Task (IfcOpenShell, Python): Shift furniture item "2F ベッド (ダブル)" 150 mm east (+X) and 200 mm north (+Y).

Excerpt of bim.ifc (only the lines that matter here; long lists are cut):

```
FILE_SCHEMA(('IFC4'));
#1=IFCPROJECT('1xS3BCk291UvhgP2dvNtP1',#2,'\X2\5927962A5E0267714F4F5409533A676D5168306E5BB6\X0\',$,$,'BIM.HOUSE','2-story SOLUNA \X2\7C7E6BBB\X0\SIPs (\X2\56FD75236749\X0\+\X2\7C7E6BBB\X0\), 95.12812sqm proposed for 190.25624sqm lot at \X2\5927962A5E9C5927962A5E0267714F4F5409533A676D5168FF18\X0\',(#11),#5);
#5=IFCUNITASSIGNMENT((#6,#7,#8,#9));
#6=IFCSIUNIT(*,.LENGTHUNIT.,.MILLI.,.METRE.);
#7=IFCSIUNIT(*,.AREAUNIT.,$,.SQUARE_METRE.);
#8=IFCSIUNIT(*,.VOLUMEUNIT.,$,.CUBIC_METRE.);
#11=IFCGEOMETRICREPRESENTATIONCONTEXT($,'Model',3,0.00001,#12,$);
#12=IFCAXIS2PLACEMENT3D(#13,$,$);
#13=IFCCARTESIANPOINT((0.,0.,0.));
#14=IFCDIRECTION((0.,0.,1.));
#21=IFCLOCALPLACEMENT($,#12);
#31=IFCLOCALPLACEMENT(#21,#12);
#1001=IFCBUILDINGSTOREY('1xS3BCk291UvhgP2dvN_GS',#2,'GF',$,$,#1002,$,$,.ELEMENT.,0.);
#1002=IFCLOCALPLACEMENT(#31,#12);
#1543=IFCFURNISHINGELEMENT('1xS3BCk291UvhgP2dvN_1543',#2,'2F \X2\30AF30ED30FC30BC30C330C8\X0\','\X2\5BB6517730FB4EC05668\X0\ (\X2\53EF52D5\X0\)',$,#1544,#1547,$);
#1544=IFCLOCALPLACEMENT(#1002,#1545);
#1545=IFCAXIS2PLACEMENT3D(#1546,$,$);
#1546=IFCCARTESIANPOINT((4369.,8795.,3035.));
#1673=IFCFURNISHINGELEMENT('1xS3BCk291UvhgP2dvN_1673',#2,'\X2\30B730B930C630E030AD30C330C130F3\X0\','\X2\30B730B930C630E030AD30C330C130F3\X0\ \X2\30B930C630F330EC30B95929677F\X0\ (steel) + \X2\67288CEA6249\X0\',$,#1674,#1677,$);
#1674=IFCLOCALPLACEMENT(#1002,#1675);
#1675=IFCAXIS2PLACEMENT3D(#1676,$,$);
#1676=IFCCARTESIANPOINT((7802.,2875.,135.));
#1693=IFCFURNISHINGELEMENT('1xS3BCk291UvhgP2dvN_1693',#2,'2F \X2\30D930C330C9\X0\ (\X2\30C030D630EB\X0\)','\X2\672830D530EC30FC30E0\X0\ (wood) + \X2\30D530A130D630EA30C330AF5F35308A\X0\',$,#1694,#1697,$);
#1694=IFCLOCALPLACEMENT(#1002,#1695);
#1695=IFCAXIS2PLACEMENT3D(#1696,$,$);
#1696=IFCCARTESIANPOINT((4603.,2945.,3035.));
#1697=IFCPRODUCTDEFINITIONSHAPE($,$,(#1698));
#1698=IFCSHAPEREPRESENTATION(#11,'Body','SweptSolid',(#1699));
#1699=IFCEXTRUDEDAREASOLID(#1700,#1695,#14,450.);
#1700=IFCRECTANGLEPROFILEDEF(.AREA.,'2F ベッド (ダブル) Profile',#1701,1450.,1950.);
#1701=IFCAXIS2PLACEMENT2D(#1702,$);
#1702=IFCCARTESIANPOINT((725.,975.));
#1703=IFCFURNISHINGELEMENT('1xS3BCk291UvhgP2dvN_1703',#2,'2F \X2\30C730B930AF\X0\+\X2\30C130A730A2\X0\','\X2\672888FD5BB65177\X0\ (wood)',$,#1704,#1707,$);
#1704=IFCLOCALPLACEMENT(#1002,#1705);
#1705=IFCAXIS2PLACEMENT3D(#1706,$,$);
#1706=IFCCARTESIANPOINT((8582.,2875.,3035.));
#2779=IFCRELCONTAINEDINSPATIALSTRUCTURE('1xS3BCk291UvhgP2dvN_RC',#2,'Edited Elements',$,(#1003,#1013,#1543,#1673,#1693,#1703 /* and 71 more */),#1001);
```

```python
import ifcopenshell
import ifcopenshell.api.geometry
import ifcopenshell.util.placement
import ifcopenshell.util.unit

model = ifcopenshell.open("bim.ifc")
unit_scale = ifcopenshell.util.unit.calculate_unit_scale(model)

item = model.by_guid("1xS3BCk291UvhgP2dvN_1693")
matrix = ifcopenshell.util.placement.get_local_placement(item.ObjectPlacement)
matrix[0, 3] += 0.15 / unit_scale
matrix[1, 3] += 0.2 / unit_scale
ifcopenshell.api.geometry.edit_object_placement(model, product=item, matrix=matrix, is_si=False)

print(ifcopenshell.util.placement.get_local_placement(item.ObjectPlacement).round(3) + 0.0)

model.write("bim_updated.ifc")
```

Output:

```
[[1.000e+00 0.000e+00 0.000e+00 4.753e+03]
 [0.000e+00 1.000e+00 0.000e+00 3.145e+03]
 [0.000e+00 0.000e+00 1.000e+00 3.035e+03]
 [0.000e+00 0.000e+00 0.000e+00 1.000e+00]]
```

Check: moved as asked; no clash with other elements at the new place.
